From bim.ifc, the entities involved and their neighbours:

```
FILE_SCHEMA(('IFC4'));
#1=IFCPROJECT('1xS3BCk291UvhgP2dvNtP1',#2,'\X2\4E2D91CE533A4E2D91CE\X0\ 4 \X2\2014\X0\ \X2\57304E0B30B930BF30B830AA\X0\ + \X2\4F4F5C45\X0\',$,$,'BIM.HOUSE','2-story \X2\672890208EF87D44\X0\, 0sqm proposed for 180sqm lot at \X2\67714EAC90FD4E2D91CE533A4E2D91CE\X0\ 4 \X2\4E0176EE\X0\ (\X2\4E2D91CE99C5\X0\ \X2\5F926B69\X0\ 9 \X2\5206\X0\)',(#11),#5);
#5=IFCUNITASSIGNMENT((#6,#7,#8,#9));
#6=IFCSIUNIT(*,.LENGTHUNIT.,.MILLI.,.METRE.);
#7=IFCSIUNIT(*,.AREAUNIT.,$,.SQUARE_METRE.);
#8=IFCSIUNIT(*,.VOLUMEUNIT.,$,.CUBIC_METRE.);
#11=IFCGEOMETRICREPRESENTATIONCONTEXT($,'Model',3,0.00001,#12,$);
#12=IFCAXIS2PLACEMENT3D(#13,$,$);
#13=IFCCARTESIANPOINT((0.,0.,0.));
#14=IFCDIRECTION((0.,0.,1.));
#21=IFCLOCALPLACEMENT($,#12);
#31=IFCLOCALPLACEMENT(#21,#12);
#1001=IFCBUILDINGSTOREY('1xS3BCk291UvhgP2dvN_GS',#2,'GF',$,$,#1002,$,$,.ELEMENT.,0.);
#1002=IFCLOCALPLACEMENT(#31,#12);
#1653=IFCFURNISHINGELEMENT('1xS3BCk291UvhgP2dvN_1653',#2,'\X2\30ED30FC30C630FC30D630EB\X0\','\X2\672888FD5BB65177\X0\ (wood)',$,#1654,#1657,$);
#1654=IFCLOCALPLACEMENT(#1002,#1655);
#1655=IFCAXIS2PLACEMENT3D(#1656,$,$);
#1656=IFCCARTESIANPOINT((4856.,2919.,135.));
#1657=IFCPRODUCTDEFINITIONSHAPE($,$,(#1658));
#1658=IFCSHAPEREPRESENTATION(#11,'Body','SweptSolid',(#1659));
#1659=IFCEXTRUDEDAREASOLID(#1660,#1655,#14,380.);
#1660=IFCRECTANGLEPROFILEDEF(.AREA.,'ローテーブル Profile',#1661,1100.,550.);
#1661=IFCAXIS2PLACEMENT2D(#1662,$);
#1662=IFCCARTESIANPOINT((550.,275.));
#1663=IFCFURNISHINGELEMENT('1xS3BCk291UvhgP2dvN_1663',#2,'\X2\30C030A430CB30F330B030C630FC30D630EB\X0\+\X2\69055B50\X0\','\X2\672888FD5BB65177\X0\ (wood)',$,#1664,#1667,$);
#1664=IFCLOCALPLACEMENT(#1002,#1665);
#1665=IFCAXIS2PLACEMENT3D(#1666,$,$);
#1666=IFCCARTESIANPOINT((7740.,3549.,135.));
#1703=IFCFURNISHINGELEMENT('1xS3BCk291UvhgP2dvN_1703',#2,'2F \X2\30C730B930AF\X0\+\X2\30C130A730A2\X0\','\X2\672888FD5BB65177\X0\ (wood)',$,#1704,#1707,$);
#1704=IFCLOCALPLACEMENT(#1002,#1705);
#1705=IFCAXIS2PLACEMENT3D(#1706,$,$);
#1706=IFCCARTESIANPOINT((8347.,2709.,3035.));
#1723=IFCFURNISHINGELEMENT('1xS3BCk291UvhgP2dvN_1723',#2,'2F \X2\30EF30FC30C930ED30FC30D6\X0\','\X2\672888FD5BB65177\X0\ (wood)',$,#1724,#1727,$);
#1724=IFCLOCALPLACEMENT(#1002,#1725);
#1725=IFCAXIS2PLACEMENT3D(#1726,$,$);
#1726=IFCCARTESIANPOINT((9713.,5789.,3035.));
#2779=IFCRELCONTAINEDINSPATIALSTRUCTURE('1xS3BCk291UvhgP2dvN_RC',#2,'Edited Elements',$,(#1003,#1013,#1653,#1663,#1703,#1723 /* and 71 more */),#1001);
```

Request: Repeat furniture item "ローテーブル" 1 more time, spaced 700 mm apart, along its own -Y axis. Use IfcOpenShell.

```python
import ifcopenshell
import ifcopenshell.api.geometry
import ifcopenshell.api.root
import ifcopenshell.util.element
import ifcopenshell.util.placement
import ifcopenshell.util.unit

model = ifcopenshell.open("bim.ifc")
unit_scale = ifcopenshell.util.unit.calculate_unit_scale(model)


def reuse_history(source, copy):
    """copy_class also copies each property set's owner history, people and application; keep the originals."""
    for rel in copy.IsDefinedBy:
        if rel.is_a("IfcRelDefinesByProperties") and (history := rel.RelatingPropertyDefinition.OwnerHistory):
            rel.RelatingPropertyDefinition.OwnerHistory = source.OwnerHistory
            ifcopenshell.util.element.remove_deep2(model, history)


source = model.by_guid("1xS3BCk291UvhgP2dvN_1653")
base = ifcopenshell.util.placement.get_local_placement(source.ObjectPlacement)
step = -base[:3, 1] * 0.7 / unit_scale

for i in range(1, 2):
    copy = ifcopenshell.api.root.copy_class(model, product=source)
    copy.Representation = ifcopenshell.util.element.copy_deep(
        model, source.Representation, exclude=["IfcGeometricRepresentationContext", "IfcRepresentationMap"]
    )
    reuse_history(source, copy)
    matrix = base.copy()
    matrix[:3, 3] += i * step
    print("added at", matrix[:3, 3].round(3) + 0.0)
    ifcopenshell.api.geometry.edit_object_placement(model, product=copy, matrix=matrix, is_si=False)

model.write("bim_rev.ifc")
```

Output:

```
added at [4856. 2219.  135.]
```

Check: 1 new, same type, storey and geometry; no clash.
